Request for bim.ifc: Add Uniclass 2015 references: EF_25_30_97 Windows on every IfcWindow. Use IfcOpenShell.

First a look at what the model holds.

```python
import ifcopenshell

model = ifcopenshell.open("bim.ifc")
print(model.schema)
print("classifications:", [c.Name for c in model.by_type("IfcClassification")])
for ifc_class in ("IfcDoor", "IfcRoof", "IfcStair", "IfcWall", "IfcWindow"):
    print(ifc_class, len(model.by_type(ifc_class)))
```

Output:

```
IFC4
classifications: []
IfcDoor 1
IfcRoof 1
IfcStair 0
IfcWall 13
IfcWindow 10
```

```python
import ifcopenshell
import ifcopenshell.api.classification

model = ifcopenshell.open("bim.ifc")

system = ifcopenshell.api.classification.add_classification(model, classification="Uniclass 2015")

codes = {
    "IfcWindow": ("EF_25_30_97", "Windows"),
}
for ifc_class, (code, name) in codes.items():
    products = model.by_type(ifc_class)
    ifcopenshell.api.classification.add_reference(
        model, products=products, classification=system, identification=code, name=name
    )
    print(code, len(products))

model.write("bim_v2.ifc")
```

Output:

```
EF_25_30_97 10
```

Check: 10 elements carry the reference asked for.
